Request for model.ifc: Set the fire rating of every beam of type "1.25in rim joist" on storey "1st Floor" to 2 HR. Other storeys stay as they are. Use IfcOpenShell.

First a look at what the model holds.

```python
import ifcopenshell
import ifcopenshell.util.element

model = ifcopenshell.open("model.ifc")
print(model.schema)
storey = next(s for s in model.by_type("IfcBuildingStorey") if s.Name == "1st Floor")
beams = [e for e in ifcopenshell.util.element.get_decomposition(storey) if e.is_a("IfcBeam")]
seen = {}
for e in beams:
    element_type = ifcopenshell.util.element.get_type(e)
    key = (element_type.Name if element_type != e and element_type else None, ifcopenshell.util.element.get_pset(e, "Pset_BeamCommon", "FireRating"))
    seen[key] = seen.get(key, 0) + 1
for (name, value), count in sorted(seen.items(), key=str):
    print(count, "x", name, "|", value)
```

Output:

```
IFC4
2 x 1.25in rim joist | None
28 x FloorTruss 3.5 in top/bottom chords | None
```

```python
import ifcopenshell
import ifcopenshell.api.pset
import ifcopenshell.util.element

model = ifcopenshell.open("model.ifc")

storey = next(s for s in model.by_type("IfcBuildingStorey") if s.Name == "1st Floor")
beams = [e for e in ifcopenshell.util.element.get_decomposition(storey) if e.is_a("IfcBeam")]

count = 0
for e in beams:
    element_type = ifcopenshell.util.element.get_type(e)
    if element_type in (None, e) or element_type.Name != "1.25in rim joist":
        continue
    # add_pset returns the element's existing set when there is one.
    pset = ifcopenshell.api.pset.add_pset(model, product=e, name="Pset_BeamCommon")
    ifcopenshell.api.pset.edit_pset(model, pset=pset, properties={"FireRating": "2 HR"})
    count += 1

print(count, "beams updated")

model.write("model_v2.ifc")
```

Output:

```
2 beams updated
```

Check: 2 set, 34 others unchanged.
